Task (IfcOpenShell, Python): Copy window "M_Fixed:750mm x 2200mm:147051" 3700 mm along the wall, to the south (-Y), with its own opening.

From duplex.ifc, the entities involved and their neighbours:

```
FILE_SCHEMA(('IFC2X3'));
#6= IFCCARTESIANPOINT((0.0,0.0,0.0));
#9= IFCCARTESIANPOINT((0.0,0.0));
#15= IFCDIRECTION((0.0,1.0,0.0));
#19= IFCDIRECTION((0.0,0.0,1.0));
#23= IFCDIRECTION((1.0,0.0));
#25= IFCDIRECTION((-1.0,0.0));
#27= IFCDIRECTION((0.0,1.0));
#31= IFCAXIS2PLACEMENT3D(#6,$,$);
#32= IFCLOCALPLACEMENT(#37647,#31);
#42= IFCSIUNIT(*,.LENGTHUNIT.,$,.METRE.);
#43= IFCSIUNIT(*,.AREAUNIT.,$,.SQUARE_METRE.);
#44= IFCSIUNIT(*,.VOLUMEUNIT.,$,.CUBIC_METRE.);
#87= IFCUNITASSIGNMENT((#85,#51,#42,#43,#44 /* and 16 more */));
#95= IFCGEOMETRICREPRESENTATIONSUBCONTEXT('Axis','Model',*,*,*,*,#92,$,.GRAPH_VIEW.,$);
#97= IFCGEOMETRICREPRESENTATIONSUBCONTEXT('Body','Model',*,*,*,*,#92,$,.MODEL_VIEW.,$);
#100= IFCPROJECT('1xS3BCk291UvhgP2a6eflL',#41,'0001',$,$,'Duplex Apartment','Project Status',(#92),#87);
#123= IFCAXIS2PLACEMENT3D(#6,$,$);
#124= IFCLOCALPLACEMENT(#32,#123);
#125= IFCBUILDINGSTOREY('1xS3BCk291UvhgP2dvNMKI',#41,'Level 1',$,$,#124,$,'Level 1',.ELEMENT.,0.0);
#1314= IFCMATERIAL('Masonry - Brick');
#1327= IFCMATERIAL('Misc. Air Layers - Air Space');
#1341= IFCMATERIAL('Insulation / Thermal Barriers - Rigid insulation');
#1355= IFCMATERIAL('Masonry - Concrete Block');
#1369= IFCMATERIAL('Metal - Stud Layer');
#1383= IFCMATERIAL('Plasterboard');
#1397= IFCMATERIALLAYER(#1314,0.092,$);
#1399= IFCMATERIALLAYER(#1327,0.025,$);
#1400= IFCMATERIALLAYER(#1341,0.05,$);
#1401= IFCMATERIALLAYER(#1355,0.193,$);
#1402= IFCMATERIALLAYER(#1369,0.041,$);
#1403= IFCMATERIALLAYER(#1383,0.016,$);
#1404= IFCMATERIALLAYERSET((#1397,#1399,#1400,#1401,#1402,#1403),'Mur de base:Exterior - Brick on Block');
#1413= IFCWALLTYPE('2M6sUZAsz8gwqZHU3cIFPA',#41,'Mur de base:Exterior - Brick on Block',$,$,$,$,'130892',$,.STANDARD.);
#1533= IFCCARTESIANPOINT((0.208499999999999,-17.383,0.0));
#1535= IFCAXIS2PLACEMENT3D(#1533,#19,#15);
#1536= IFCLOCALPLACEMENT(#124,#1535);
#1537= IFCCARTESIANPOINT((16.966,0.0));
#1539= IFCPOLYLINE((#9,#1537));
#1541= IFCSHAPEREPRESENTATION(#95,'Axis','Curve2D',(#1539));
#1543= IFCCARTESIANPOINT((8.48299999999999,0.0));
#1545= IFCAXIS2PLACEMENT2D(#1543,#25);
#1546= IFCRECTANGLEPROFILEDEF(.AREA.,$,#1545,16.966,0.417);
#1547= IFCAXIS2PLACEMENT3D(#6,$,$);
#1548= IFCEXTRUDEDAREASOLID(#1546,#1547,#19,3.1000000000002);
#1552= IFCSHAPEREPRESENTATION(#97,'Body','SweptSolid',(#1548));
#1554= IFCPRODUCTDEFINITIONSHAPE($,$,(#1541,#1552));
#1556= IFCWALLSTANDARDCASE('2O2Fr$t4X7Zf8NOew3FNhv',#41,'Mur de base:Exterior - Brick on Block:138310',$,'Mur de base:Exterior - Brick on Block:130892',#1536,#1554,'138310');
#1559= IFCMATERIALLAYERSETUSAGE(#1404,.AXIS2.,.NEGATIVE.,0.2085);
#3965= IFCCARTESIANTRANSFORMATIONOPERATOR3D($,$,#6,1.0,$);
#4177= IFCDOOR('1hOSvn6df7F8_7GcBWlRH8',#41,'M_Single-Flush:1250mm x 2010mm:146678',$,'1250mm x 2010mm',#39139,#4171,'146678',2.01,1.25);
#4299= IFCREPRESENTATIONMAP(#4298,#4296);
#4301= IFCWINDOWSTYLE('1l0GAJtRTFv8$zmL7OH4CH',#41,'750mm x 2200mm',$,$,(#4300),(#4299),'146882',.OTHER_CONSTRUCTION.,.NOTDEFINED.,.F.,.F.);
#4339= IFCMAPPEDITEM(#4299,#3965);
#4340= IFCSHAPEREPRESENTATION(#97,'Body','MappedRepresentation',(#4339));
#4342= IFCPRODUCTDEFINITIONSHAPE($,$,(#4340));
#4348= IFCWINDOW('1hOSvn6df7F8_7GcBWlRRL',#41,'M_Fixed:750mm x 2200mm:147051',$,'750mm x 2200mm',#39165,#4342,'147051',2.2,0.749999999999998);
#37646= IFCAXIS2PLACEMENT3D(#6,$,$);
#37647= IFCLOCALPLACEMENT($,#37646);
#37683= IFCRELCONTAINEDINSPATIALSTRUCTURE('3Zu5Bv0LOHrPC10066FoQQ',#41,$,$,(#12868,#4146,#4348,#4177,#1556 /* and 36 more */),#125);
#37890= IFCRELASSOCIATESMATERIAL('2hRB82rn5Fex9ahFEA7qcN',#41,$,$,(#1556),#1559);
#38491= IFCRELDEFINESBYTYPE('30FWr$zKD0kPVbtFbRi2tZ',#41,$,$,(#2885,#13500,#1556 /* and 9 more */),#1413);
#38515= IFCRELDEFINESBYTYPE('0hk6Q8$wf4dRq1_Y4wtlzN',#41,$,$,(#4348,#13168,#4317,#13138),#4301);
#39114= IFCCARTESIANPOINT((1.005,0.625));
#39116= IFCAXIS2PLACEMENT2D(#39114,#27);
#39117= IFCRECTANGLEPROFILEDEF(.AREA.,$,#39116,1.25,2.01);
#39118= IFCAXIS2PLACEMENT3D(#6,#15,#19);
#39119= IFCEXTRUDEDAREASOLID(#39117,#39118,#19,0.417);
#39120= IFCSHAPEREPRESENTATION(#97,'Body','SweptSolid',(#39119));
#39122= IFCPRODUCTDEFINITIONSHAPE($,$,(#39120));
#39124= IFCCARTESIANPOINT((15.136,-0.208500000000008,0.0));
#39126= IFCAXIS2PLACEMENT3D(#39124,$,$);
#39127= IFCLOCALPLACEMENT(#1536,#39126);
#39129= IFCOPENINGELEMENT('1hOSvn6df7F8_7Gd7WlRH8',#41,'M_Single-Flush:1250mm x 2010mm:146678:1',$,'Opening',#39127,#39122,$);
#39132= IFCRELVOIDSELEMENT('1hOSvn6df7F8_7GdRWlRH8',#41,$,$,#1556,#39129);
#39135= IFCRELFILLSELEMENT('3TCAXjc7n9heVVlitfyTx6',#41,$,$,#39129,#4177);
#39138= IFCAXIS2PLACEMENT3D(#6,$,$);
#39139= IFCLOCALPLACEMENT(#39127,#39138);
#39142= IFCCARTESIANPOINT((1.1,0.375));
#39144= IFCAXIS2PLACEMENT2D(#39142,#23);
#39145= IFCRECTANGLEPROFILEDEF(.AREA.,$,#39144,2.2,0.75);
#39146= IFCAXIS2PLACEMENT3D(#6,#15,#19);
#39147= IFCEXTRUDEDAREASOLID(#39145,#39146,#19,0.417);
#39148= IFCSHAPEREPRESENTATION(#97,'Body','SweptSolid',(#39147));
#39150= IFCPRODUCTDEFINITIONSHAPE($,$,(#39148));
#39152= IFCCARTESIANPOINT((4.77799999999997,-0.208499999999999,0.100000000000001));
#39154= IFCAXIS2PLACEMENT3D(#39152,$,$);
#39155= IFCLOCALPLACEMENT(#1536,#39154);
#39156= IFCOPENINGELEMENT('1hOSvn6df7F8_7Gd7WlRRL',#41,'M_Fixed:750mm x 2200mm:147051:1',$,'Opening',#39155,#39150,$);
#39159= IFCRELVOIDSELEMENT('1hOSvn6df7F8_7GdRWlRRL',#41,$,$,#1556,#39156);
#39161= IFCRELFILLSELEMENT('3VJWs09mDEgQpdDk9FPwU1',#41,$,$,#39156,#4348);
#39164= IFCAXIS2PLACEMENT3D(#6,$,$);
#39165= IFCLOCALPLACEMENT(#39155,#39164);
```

```python
import ifcopenshell
import ifcopenshell.api.feature
import ifcopenshell.api.geometry
import ifcopenshell.api.root
import ifcopenshell.geom
import ifcopenshell.util.element
import ifcopenshell.util.placement
import ifcopenshell.util.shape
import ifcopenshell.util.unit

model = ifcopenshell.open("duplex.ifc")
unit_scale = ifcopenshell.util.unit.calculate_unit_scale(model)
settings = ifcopenshell.geom.settings()


def volume(element):
    """Net volume in cubic metres, openings subtracted."""
    shape = ifcopenshell.geom.create_shape(settings, element)
    return ifcopenshell.util.shape.get_volume(shape.geometry)


def reuse_history(source, copy):
    """copy_class also copies each property set's owner history, people and application; keep the originals."""
    for rel in copy.IsDefinedBy:
        if rel.is_a("IfcRelDefinesByProperties") and (history := rel.RelatingPropertyDefinition.OwnerHistory):
            rel.RelatingPropertyDefinition.OwnerHistory = source.OwnerHistory
            ifcopenshell.util.element.remove_deep2(model, history)


window = model.by_id(4348)
opening = window.FillsVoids[0].RelatingOpeningElement
wall = opening.VoidsElements[0].RelatingBuildingElement
before = volume(wall)
shift = ifcopenshell.util.placement.get_local_placement(wall.ObjectPlacement)[:3, 0] * -3.7 / unit_scale

# copy_class copies the void relationship, type, container and properties, but no geometry.
new_opening = ifcopenshell.api.root.copy_class(model, product=opening)
new_opening.Representation = ifcopenshell.util.element.copy_deep(
    model, opening.Representation, exclude=["IfcGeometricRepresentationContext", "IfcRepresentationMap"]
)
new_opening.Name = "M_Fixed:750mm x 2200mm"
new_window = ifcopenshell.api.root.copy_class(model, product=window)
new_window.Representation = ifcopenshell.util.element.copy_deep(
    model, window.Representation, exclude=["IfcGeometricRepresentationContext", "IfcRepresentationMap"]
)
new_window.Name = "M_Fixed:750mm x 2200mm"
new_window.Tag = None
reuse_history(window, new_window)
fills = ifcopenshell.api.feature.add_filling(model, opening=new_opening, element=new_window)
fills.OwnerHistory = new_window.OwnerHistory  # required in IFC2X3

for old, new in ((opening, new_opening), (window, new_window)):
    matrix = ifcopenshell.util.placement.get_local_placement(old.ObjectPlacement)
    matrix[:3, 3] += shift
    ifcopenshell.api.geometry.edit_object_placement(model, product=new, matrix=matrix, is_si=False)

after = volume(wall)

print(f"wall volume {before:.3f} -> {after:.3f} m3")

model.write("duplex_rev.ifc")
```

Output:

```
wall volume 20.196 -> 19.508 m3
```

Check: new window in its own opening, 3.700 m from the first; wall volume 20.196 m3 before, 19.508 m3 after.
